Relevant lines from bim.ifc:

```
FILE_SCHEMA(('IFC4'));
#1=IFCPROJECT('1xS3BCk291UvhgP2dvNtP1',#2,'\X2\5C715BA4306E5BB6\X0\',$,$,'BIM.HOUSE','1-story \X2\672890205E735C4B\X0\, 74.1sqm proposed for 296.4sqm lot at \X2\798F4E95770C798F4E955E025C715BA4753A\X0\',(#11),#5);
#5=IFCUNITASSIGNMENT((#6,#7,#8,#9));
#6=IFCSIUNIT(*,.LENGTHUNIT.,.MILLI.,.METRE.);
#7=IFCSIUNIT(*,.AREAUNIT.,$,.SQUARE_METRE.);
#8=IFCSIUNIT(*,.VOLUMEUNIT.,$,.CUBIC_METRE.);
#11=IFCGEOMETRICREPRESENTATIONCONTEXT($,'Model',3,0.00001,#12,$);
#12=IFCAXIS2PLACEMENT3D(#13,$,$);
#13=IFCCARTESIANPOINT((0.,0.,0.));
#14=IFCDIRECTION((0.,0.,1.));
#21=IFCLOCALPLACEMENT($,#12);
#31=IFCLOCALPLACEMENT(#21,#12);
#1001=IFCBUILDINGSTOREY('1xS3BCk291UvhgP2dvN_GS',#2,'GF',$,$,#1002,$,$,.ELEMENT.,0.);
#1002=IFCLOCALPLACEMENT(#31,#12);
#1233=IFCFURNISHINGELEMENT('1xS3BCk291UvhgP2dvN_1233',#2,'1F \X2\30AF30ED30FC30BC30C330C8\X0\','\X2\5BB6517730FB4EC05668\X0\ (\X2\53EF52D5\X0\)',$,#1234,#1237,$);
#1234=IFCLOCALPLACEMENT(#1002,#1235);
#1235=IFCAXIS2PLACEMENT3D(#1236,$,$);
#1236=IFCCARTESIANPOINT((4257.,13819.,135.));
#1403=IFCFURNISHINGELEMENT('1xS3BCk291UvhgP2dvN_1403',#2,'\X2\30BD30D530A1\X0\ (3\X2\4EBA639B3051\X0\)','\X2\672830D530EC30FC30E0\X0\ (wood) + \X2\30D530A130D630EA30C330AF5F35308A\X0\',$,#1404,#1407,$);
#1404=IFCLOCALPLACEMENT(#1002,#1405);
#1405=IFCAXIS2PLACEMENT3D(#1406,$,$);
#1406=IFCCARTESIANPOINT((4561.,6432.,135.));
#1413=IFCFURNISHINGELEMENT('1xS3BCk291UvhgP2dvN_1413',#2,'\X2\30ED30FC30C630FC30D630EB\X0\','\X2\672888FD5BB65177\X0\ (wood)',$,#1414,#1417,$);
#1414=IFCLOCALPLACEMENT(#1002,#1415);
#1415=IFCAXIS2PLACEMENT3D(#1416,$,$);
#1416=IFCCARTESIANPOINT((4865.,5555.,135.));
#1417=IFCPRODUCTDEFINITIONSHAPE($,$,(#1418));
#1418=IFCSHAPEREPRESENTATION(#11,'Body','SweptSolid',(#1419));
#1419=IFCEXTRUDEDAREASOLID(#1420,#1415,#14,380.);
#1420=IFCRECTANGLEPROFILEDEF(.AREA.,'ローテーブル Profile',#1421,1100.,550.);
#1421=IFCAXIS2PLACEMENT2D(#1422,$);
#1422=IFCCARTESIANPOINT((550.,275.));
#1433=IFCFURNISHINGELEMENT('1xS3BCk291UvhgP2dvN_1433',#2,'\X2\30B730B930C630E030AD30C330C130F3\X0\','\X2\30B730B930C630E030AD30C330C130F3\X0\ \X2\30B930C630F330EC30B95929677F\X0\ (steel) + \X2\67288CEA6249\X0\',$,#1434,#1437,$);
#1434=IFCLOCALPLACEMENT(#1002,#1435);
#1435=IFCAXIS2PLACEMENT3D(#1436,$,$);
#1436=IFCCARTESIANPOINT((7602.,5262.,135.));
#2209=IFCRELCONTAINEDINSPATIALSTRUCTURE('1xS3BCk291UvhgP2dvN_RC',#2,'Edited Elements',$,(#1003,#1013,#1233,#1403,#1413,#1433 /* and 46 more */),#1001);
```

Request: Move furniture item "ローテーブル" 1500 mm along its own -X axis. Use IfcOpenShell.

```python
import ifcopenshell
import ifcopenshell.api.geometry
import ifcopenshell.util.placement

model = ifcopenshell.open("bim.ifc")

item = model.by_guid("1xS3BCk291UvhgP2dvN_1413")
matrix = ifcopenshell.util.placement.get_local_placement(item.ObjectPlacement)
matrix[:3, 3] -= matrix[:3, 0] * 1500.0
ifcopenshell.api.geometry.edit_object_placement(model, product=item, matrix=matrix, is_si=False)

print(ifcopenshell.util.placement.get_local_placement(item.ObjectPlacement).round(3) + 0.0)

model.write("bim_rev.ifc")
```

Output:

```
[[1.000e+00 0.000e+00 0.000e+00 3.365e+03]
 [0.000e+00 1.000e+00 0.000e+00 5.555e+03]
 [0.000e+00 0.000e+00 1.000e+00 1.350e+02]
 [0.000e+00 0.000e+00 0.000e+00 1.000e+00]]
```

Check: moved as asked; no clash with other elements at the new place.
